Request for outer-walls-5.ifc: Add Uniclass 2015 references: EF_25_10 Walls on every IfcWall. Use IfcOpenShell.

First a look at what the model holds.

```python
import ifcopenshell

model = ifcopenshell.open("outer-walls-5.ifc")
print(model.schema)
print("classifications:", [c.Name for c in model.by_type("IfcClassification")])
for ifc_class in ("IfcDoor", "IfcRoof", "IfcStair", "IfcWall", "IfcWindow"):
    print(ifc_class, len(model.by_type(ifc_class)))
```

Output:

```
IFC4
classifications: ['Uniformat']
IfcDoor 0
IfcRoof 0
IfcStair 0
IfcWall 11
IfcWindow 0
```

```python
import ifcopenshell
import ifcopenshell.api.classification

model = ifcopenshell.open("outer-walls-5.ifc")

system = ifcopenshell.api.classification.add_classification(model, classification="Uniclass 2015")

codes = {
    "IfcWall": ("EF_25_10", "Walls"),
}
for ifc_class, (code, name) in codes.items():
    products = model.by_type(ifc_class)
    ifcopenshell.api.classification.add_reference(
        model, products=products, classification=system, identification=code, name=name
    )
    print(code, len(products))

model.write("outer-walls-5_v2.ifc")
```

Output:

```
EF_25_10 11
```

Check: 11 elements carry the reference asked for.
